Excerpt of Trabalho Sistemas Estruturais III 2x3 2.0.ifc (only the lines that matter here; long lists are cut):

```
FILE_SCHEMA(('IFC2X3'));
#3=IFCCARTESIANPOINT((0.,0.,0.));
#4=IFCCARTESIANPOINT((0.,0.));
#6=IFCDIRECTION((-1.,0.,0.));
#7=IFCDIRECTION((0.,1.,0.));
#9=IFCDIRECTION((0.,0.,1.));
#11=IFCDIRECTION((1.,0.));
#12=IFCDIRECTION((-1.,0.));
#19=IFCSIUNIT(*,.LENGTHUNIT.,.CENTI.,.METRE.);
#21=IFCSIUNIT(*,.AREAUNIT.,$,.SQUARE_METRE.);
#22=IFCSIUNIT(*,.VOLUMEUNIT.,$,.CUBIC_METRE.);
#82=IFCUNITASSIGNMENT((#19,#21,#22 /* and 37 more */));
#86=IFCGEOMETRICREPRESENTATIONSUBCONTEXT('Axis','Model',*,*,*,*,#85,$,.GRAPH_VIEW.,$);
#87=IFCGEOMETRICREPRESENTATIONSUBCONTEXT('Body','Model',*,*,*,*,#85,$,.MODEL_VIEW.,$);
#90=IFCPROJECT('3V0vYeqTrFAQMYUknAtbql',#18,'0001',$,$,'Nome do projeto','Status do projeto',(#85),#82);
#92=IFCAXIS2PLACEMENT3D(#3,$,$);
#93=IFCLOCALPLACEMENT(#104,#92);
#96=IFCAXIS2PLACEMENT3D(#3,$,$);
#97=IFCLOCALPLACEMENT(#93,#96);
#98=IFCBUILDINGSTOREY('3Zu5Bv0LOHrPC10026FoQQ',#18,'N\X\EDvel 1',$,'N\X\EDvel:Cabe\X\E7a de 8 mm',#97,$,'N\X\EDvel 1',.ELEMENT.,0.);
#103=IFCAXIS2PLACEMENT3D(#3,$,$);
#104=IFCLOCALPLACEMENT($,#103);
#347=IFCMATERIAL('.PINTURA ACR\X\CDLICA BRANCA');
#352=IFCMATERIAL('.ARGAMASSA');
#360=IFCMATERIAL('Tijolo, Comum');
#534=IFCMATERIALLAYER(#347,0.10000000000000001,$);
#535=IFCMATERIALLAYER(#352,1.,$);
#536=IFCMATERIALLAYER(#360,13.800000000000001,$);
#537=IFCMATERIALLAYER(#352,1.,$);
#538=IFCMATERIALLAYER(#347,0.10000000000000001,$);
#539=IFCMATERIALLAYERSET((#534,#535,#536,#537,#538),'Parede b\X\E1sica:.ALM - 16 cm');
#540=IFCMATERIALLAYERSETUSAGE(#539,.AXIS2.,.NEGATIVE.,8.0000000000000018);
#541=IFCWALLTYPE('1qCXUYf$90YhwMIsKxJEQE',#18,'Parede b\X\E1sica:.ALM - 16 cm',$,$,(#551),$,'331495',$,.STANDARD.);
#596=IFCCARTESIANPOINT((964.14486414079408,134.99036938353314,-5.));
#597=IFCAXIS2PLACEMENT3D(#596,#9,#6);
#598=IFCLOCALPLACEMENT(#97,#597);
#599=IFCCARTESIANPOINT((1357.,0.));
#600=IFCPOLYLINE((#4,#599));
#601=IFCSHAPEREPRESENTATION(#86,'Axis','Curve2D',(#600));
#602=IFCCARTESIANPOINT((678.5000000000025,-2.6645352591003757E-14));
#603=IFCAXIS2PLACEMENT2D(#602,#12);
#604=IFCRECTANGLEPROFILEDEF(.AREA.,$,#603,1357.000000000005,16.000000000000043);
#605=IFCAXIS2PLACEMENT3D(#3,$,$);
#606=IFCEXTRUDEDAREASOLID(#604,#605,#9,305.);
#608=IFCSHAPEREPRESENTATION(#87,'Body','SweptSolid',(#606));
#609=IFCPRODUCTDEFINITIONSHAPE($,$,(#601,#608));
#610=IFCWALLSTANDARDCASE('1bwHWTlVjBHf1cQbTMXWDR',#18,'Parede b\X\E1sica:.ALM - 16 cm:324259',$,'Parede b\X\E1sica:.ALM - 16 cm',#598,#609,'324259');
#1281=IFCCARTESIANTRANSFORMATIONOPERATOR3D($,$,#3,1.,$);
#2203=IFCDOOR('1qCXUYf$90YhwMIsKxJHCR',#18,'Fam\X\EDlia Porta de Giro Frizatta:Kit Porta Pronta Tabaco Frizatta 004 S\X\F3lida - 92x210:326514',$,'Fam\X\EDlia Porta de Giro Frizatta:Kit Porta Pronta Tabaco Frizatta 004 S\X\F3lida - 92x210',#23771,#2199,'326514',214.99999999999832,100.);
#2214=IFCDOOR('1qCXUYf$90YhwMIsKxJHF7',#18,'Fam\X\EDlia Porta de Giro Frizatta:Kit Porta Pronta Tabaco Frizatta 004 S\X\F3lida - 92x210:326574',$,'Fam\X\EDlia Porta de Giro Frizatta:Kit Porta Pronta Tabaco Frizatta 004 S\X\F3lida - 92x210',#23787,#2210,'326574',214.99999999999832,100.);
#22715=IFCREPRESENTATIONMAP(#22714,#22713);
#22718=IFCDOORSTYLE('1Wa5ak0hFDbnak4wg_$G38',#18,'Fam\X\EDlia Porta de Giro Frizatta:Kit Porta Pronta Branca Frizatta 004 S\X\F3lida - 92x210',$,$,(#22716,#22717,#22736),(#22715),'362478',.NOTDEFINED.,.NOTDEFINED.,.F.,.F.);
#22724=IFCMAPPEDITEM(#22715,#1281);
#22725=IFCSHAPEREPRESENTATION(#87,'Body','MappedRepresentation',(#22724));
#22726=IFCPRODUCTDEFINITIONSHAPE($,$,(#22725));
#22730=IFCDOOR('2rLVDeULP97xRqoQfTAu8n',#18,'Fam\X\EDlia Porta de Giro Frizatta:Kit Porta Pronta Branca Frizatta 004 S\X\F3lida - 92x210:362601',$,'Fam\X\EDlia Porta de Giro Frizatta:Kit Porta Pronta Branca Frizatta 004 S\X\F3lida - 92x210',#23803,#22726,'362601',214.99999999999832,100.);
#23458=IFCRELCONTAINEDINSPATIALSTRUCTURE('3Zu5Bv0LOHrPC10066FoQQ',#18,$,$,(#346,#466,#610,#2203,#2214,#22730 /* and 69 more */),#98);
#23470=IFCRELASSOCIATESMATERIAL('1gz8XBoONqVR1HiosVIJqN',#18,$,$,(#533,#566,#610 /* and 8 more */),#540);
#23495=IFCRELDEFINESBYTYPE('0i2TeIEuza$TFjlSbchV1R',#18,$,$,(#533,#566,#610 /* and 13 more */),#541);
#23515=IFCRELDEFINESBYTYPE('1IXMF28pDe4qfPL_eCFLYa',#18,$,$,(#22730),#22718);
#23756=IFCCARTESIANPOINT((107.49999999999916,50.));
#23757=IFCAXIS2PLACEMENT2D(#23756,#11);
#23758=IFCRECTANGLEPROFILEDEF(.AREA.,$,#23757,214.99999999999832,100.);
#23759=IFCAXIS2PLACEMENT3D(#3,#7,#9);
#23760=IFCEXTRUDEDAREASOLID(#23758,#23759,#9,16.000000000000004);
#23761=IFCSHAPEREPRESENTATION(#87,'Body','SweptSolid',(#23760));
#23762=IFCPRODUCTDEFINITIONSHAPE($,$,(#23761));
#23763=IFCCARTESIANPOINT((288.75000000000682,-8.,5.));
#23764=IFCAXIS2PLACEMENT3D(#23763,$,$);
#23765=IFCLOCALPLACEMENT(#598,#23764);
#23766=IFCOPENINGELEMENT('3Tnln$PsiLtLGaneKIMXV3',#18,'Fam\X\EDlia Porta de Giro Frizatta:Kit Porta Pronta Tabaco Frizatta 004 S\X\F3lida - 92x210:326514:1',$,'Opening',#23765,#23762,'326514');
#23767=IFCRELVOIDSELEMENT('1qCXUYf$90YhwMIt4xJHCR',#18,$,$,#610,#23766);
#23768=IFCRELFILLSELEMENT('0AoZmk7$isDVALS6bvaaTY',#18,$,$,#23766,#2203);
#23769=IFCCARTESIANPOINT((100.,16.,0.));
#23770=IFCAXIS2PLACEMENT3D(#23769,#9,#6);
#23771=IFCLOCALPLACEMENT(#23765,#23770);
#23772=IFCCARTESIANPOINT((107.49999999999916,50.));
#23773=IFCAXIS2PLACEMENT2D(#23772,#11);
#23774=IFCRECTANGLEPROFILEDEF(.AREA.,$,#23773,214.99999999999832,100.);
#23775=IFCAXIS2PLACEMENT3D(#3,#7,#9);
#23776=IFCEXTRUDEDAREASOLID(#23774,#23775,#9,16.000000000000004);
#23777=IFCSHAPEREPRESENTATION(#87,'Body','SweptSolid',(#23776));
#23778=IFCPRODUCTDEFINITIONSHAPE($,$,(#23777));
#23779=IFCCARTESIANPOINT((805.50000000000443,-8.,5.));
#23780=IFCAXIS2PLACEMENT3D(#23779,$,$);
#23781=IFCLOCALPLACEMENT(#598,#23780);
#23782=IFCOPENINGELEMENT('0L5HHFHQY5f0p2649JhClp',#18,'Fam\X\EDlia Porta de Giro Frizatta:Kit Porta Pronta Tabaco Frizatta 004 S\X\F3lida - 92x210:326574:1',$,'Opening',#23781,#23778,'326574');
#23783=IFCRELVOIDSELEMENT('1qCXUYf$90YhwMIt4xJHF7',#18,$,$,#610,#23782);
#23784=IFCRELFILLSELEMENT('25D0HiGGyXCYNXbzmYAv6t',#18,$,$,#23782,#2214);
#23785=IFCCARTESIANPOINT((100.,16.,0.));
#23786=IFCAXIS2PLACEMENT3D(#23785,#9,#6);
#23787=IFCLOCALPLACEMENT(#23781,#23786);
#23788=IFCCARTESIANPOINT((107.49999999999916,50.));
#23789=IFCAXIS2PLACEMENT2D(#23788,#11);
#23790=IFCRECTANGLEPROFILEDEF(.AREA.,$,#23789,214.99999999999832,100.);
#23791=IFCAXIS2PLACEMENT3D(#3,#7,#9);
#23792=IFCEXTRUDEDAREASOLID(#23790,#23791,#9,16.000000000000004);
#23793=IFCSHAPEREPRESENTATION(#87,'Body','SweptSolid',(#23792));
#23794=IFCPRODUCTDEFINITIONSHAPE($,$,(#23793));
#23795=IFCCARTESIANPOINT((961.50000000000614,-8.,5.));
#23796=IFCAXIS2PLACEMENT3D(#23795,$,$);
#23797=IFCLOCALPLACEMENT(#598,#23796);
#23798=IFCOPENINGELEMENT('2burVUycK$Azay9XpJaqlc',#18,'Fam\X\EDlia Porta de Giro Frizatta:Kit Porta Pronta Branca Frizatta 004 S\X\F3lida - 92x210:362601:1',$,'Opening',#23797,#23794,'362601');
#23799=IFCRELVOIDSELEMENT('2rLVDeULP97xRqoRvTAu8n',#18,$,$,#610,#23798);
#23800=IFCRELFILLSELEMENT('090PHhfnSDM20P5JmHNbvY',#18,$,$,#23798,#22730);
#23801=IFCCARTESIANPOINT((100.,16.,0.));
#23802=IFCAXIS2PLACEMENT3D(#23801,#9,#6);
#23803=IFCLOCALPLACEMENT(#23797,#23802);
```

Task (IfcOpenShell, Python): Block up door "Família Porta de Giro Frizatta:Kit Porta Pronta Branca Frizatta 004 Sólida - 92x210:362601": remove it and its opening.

```python
import ifcopenshell
import ifcopenshell.api.feature
import ifcopenshell.api.root
import ifcopenshell.geom
import ifcopenshell.util.shape

model = ifcopenshell.open("Trabalho Sistemas Estruturais III 2x3 2.0.ifc")
settings = ifcopenshell.geom.settings()


def volume(element):
    """Net volume in cubic metres, openings subtracted."""
    shape = ifcopenshell.geom.create_shape(settings, element)
    return ifcopenshell.util.shape.get_volume(shape.geometry)


door = model.by_guid("2rLVDeULP97xRqoQfTAu8n")
opening = door.FillsVoids[0].RelatingOpeningElement
wall = opening.VoidsElements[0].RelatingBuildingElement
before = volume(wall)

ifcopenshell.api.root.remove_product(model, product=door)
ifcopenshell.api.feature.remove_feature(model, feature=opening)

after = volume(wall)

print(f"wall volume {before:.3f} -> {after:.3f} m3")

model.write("Trabalho Sistemas Estruturais III 2x3 2.0-out.ifc")
```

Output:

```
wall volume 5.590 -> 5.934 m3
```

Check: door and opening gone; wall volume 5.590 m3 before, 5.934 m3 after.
